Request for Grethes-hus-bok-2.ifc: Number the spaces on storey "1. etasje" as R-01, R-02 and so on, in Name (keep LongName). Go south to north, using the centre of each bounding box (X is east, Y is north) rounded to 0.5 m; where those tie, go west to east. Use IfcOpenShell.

First a look at what the model holds.

```python
import ifcopenshell
import ifcopenshell.util.element
import ifcopenshell.util.placement

model = ifcopenshell.open("Grethes-hus-bok-2.ifc")
print(model.schema)
storey = next(s for s in model.by_type("IfcBuildingStorey") if s.Name == "1. etasje")
spaces = [e for e in ifcopenshell.util.element.get_decomposition(storey) if e.is_a("IfcSpace")]
for e in sorted(spaces, key=lambda e: e.id()):
    origin = ifcopenshell.util.placement.get_local_placement(e.ObjectPlacement)[:3, 3]
    print(e.id(), e.Name, e.LongName, origin.round(2) + 0.0, sep=" | ")
```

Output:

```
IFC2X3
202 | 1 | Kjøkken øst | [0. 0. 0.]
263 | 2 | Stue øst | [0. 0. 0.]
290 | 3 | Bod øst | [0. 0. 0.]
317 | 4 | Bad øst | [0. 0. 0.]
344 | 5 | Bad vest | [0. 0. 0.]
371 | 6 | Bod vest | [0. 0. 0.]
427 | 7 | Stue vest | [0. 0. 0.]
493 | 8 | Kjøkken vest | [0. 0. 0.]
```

```python
import ifcopenshell
import ifcopenshell.geom
import ifcopenshell.util.element
import ifcopenshell.util.shape

model = ifcopenshell.open("Grethes-hus-bok-2.ifc")
settings = ifcopenshell.geom.settings()
settings.set("use-world-coords", True)


def centre(element):
    shape = ifcopenshell.geom.create_shape(settings, element)
    return ifcopenshell.util.shape.get_bbox_centroid(shape.geometry)


storey = next(s for s in model.by_type("IfcBuildingStorey") if s.Name == "1. etasje")
spaces = [e for e in ifcopenshell.util.element.get_decomposition(storey) if e.is_a("IfcSpace")]

# Insertion points can sit at a corner or the storey origin, so sort by the geometry (in metres).
centres = {e: centre(e) for e in spaces}
spaces.sort(key=lambda e: (round(centres[e][1] / 0.5), centres[e][0]))

for i, e in enumerate(spaces, start=1):
    number = f"R-{i:02d}"
    e.Name = number
    print(e.id(), number)

model.write("Grethes-hus-bok-2_edited.ifc")
```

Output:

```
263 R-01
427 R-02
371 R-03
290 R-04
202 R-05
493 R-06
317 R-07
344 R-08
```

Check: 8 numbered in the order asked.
